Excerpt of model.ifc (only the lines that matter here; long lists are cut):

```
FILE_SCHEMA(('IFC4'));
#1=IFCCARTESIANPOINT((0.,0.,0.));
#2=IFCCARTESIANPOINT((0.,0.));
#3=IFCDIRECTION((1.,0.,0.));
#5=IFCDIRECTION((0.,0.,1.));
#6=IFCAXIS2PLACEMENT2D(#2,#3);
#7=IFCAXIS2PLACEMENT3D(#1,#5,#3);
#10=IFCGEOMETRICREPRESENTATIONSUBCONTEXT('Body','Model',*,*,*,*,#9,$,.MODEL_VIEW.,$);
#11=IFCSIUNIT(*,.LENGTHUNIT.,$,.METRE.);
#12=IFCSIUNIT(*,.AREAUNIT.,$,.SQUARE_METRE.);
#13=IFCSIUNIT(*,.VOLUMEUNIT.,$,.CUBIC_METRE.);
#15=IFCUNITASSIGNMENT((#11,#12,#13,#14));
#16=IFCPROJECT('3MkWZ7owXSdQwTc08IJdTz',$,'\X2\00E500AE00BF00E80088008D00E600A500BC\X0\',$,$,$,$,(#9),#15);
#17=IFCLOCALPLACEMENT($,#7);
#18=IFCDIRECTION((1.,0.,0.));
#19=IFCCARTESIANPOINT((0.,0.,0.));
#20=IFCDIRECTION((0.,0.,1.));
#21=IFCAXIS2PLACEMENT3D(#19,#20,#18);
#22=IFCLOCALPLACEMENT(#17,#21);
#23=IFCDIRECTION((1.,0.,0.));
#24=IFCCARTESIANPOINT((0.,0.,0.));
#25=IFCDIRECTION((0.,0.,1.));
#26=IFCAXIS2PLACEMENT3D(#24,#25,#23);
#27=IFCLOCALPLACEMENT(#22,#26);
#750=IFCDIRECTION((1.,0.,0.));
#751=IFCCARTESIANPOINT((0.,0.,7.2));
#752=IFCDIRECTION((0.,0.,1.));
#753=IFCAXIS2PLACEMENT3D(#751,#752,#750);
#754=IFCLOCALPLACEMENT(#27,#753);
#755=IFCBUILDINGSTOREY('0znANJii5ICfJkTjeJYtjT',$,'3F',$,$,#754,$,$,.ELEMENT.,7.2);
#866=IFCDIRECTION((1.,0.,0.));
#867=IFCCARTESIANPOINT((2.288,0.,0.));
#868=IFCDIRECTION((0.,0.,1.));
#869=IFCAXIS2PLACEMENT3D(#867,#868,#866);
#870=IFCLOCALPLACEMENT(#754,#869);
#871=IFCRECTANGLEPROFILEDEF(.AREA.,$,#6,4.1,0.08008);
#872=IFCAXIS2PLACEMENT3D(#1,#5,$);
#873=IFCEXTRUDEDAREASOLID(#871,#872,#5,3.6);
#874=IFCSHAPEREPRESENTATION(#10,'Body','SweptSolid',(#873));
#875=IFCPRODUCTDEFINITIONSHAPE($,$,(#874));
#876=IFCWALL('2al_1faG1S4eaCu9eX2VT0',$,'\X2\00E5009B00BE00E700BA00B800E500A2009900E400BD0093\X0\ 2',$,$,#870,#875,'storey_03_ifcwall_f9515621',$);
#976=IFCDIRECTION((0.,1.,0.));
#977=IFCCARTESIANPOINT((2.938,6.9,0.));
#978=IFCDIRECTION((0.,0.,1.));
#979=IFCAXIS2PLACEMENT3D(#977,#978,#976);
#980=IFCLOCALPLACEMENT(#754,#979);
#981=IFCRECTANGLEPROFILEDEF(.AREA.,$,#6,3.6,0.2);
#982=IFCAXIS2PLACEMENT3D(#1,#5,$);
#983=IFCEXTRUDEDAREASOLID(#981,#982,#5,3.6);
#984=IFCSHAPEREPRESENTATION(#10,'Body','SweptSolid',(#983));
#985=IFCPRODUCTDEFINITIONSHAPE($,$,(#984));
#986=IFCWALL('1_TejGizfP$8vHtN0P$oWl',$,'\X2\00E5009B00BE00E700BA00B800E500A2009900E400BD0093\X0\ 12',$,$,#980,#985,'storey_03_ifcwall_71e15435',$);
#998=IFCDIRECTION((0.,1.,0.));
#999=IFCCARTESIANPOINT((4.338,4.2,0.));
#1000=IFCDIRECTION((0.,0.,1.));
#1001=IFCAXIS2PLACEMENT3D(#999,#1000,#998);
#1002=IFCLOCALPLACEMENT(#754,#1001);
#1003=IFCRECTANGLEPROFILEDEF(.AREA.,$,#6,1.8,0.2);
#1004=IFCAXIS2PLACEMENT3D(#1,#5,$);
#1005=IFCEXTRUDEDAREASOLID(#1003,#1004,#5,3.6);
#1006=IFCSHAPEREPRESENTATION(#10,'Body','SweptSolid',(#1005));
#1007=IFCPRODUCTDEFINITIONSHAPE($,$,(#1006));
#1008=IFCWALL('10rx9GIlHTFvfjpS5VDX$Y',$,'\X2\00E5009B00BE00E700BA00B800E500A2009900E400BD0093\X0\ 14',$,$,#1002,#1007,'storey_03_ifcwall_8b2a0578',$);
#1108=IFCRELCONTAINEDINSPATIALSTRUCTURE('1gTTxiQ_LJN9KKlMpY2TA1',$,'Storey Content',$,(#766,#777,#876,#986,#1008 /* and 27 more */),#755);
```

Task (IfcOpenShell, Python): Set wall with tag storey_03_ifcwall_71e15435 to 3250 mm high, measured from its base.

```python
import ifcopenshell
import ifcopenshell.geom
import ifcopenshell.util.representation
import ifcopenshell.util.shape

model = ifcopenshell.open("model.ifc")
settings = ifcopenshell.geom.settings()


def volume(element):
    """Net volume in cubic metres, openings subtracted."""
    shape = ifcopenshell.geom.create_shape(settings, element)
    return ifcopenshell.util.shape.get_volume(shape.geometry)


wall = model.by_guid("1_TejGizfP$8vHtN0P$oWl")
before = volume(wall)

body = ifcopenshell.util.representation.get_representation(wall, "Model", "Body")
solid = body.Items[0]
old_height = solid.Depth
solid.Depth = 3.25
after = volume(wall)

print(f"height {old_height:g} -> {solid.Depth:g}, volume {before:.3f} -> {after:.3f} m3")

model.write("model_updated.ifc")
```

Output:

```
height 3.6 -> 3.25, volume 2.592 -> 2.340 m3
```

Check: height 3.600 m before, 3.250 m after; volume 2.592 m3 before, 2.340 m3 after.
